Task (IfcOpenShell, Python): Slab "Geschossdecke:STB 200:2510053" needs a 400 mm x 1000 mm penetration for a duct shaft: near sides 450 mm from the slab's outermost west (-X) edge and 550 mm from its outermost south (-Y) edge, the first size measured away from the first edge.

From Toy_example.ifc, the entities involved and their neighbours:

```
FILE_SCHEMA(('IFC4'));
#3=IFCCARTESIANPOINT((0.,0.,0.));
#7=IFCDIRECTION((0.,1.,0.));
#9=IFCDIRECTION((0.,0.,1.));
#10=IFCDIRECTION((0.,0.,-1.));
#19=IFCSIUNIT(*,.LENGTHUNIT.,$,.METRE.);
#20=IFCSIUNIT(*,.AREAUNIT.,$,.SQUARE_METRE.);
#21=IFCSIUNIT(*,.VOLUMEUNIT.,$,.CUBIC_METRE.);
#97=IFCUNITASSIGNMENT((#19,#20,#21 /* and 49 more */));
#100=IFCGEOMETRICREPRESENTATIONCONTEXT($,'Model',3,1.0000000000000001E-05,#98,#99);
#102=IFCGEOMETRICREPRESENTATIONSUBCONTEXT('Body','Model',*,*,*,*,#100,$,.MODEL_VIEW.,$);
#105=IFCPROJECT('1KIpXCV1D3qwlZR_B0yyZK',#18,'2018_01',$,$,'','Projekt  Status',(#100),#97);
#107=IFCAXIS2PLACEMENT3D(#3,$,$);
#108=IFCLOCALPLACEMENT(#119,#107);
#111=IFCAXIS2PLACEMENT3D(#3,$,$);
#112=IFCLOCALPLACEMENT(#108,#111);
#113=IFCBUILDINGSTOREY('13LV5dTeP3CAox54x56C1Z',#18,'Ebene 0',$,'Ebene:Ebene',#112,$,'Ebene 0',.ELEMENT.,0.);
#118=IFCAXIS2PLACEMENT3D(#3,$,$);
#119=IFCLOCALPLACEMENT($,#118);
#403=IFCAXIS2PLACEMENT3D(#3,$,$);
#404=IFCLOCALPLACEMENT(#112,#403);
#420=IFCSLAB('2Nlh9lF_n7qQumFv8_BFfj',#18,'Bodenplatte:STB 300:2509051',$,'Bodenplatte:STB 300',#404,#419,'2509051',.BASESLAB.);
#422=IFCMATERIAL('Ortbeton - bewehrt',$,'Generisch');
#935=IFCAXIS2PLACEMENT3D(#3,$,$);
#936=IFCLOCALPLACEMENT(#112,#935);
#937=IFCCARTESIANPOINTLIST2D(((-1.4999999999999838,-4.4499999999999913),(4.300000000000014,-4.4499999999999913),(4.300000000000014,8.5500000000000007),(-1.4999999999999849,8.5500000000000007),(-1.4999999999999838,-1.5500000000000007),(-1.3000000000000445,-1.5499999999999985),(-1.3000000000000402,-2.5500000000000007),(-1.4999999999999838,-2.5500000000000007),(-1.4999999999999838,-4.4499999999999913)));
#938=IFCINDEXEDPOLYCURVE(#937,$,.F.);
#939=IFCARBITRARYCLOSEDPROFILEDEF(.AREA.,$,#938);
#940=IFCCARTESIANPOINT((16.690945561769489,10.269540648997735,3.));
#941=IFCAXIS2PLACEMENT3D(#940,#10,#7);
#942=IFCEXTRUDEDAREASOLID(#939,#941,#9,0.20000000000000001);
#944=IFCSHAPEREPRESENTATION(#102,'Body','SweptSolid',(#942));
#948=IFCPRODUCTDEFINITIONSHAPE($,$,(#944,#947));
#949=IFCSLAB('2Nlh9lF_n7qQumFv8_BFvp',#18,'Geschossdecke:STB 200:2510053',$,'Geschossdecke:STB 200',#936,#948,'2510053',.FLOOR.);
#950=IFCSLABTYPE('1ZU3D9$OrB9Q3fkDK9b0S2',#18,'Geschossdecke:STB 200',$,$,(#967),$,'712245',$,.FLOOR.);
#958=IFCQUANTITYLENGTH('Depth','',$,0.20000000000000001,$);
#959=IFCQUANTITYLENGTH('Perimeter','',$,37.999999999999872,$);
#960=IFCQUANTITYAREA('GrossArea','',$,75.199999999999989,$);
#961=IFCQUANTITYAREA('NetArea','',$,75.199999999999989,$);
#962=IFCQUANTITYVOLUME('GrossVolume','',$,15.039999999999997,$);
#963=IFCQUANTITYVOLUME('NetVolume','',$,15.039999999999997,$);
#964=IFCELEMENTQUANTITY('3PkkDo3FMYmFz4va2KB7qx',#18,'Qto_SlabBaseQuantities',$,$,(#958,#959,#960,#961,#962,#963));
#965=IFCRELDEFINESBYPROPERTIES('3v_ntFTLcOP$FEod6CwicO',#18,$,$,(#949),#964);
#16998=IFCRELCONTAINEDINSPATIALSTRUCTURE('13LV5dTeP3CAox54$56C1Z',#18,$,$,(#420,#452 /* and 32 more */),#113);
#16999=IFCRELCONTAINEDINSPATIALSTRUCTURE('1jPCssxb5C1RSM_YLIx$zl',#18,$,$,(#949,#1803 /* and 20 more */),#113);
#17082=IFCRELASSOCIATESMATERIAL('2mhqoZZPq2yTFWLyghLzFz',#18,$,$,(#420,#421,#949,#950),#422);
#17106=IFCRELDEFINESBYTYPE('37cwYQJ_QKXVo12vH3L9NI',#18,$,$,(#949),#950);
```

```python
import numpy as np
import ifcopenshell
import ifcopenshell.api.feature
import ifcopenshell.api.geometry
import ifcopenshell.api.pset
import ifcopenshell.api.root
import ifcopenshell.geom
import ifcopenshell.util.element
import ifcopenshell.util.placement
import ifcopenshell.util.representation
import ifcopenshell.util.shape
import ifcopenshell.util.unit

model = ifcopenshell.open("Toy_example.ifc")
unit_scale = ifcopenshell.util.unit.calculate_unit_scale(model)
area_scale = ifcopenshell.util.unit.calculate_unit_scale(model, "AREAUNIT")
volume_scale = ifcopenshell.util.unit.calculate_unit_scale(model, "VOLUMEUNIT")
settings = ifcopenshell.geom.settings()


def volume(element):
    """Net volume in cubic metres, openings subtracted."""
    shape = ifcopenshell.geom.create_shape(settings, element)
    return ifcopenshell.util.shape.get_volume(shape.geometry)


slab = model.by_guid("2Nlh9lF_n7qQumFv8_BFvp")
before = volume(slab)

# Extent in the slab's own axes, in metres. The edges named are its -X and -Y sides.
slab_shape = ifcopenshell.geom.create_shape(settings, slab)
vertices = ifcopenshell.util.shape.get_vertices(slab_shape.geometry)
x_min, y_min, bottom = vertices.min(axis=0)
top = vertices[:, 2].max()

opening = ifcopenshell.api.root.create_entity(model, ifc_class="IfcOpeningElement", name="Duct shaft opening", predefined_type="OPENING")
context = ifcopenshell.util.representation.get_context(model, "Model", "Body", "MODEL_VIEW")
width, depth = 0.4, 1
outline = [(0.0, 0.0), (width, 0.0), (width, depth), (0.0, depth), (0.0, 0.0)]
# Overshoot both faces by 50 mm so the cut is clean.
shape = ifcopenshell.api.geometry.add_slab_representation(
    model, context=context, depth=top - bottom + 0.1, polyline=outline
)
ifcopenshell.api.geometry.assign_representation(model, product=opening, representation=shape)

matrix = ifcopenshell.util.placement.get_local_placement(slab.ObjectPlacement)
matrix[:, 3] = matrix @ np.append(np.array([x_min + 0.45, y_min + 0.55, bottom - 0.05]) / unit_scale, 1.0)
ifcopenshell.api.geometry.edit_object_placement(model, product=opening, matrix=matrix, is_si=False)
ifcopenshell.api.feature.add_feature(model, feature=opening, element=slab)

after = volume(slab)

# Update the slab's stored quantities.
qto = model.by_id(ifcopenshell.util.element.get_pset(slab, "Qto_SlabBaseQuantities", should_inherit=False)["id"])
ifcopenshell.api.pset.edit_qto(model, qto=qto, properties={
    "NetArea": after / (top - bottom) / area_scale,
    "NetVolume": after / volume_scale,
})

print(f"slab volume {before:.3f} -> {after:.3f} m3")

model.write("Toy_example_edited.ifc")
```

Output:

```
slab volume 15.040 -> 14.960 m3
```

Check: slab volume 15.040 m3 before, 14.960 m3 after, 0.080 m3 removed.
